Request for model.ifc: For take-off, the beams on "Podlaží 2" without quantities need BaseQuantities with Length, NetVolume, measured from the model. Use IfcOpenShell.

First a look at what the model holds.

```python
import ifcopenshell
import ifcopenshell.util.element
import ifcopenshell.util.unit

model = ifcopenshell.open("model.ifc")
print(model.schema)
for unit_type in ("LENGTHUNIT", "AREAUNIT", "VOLUMEUNIT"):
    print(unit_type, ifcopenshell.util.unit.calculate_unit_scale(model, unit_type))
storey = next(s for s in model.by_type("IfcBuildingStorey") if s.Name == "Podlaží 2")
beams = [e for e in ifcopenshell.util.element.get_decomposition(storey) if e.is_a("IfcBeam")]
for e in sorted(beams, key=lambda e: e.id()):
    print(e.id(), e.is_a(), e.Name, list(ifcopenshell.util.element.get_psets(e, qtos_only=True)), sep=" | ")
```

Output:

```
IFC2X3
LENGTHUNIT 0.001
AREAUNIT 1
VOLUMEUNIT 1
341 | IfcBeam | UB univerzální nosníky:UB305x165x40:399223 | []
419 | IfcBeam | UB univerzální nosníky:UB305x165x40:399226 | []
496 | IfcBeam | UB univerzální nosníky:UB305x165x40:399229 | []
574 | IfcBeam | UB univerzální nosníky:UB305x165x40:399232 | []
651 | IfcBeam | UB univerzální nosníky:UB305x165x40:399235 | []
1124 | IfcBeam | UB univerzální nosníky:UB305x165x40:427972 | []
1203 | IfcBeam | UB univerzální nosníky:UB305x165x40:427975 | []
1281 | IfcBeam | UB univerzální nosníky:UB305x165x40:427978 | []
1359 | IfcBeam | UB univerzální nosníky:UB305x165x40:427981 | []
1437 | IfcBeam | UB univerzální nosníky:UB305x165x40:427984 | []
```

```python
import ifcopenshell
import ifcopenshell.api.pset
import ifcopenshell.geom
import ifcopenshell.util.element
import ifcopenshell.util.shape
import ifcopenshell.util.unit

model = ifcopenshell.open("model.ifc")
unit_scale = ifcopenshell.util.unit.calculate_unit_scale(model)
volume_scale = ifcopenshell.util.unit.calculate_unit_scale(model, "VOLUMEUNIT")
settings = ifcopenshell.geom.settings()

storey = next(s for s in model.by_type("IfcBuildingStorey") if s.Name == "Podlaží 2")
beams = [e for e in ifcopenshell.util.element.get_decomposition(storey) if e.is_a("IfcBeam")]

for e in sorted(beams, key=lambda e: e.id()):
    if ifcopenshell.util.element.get_psets(e, qtos_only=True, should_inherit=False):
        continue
    # Geometry comes back in metres, in the element's own axes.
    shape = ifcopenshell.geom.create_shape(settings, e)
    values = {
        "Length": ifcopenshell.util.shape.get_max_xyz(shape.geometry) / unit_scale,
        "NetVolume": ifcopenshell.util.shape.get_volume(shape.geometry) / volume_scale,
    }
    qto = ifcopenshell.api.pset.add_qto(model, product=e, name="BaseQuantities")
    ifcopenshell.api.pset.edit_qto(model, qto=qto, properties=values)
    print(e.id(), {k: round(v, 3) for k, v in values.items()})

model.write("model_v2.ifc")
```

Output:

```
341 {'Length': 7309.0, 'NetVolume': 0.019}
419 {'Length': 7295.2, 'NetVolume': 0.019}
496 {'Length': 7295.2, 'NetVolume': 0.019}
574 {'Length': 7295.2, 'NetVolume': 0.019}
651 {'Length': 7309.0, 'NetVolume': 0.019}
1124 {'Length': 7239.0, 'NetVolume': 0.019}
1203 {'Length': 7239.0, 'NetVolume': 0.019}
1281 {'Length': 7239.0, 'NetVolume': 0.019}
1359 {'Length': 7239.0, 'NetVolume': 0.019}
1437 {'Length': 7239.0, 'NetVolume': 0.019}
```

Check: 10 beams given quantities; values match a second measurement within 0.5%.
